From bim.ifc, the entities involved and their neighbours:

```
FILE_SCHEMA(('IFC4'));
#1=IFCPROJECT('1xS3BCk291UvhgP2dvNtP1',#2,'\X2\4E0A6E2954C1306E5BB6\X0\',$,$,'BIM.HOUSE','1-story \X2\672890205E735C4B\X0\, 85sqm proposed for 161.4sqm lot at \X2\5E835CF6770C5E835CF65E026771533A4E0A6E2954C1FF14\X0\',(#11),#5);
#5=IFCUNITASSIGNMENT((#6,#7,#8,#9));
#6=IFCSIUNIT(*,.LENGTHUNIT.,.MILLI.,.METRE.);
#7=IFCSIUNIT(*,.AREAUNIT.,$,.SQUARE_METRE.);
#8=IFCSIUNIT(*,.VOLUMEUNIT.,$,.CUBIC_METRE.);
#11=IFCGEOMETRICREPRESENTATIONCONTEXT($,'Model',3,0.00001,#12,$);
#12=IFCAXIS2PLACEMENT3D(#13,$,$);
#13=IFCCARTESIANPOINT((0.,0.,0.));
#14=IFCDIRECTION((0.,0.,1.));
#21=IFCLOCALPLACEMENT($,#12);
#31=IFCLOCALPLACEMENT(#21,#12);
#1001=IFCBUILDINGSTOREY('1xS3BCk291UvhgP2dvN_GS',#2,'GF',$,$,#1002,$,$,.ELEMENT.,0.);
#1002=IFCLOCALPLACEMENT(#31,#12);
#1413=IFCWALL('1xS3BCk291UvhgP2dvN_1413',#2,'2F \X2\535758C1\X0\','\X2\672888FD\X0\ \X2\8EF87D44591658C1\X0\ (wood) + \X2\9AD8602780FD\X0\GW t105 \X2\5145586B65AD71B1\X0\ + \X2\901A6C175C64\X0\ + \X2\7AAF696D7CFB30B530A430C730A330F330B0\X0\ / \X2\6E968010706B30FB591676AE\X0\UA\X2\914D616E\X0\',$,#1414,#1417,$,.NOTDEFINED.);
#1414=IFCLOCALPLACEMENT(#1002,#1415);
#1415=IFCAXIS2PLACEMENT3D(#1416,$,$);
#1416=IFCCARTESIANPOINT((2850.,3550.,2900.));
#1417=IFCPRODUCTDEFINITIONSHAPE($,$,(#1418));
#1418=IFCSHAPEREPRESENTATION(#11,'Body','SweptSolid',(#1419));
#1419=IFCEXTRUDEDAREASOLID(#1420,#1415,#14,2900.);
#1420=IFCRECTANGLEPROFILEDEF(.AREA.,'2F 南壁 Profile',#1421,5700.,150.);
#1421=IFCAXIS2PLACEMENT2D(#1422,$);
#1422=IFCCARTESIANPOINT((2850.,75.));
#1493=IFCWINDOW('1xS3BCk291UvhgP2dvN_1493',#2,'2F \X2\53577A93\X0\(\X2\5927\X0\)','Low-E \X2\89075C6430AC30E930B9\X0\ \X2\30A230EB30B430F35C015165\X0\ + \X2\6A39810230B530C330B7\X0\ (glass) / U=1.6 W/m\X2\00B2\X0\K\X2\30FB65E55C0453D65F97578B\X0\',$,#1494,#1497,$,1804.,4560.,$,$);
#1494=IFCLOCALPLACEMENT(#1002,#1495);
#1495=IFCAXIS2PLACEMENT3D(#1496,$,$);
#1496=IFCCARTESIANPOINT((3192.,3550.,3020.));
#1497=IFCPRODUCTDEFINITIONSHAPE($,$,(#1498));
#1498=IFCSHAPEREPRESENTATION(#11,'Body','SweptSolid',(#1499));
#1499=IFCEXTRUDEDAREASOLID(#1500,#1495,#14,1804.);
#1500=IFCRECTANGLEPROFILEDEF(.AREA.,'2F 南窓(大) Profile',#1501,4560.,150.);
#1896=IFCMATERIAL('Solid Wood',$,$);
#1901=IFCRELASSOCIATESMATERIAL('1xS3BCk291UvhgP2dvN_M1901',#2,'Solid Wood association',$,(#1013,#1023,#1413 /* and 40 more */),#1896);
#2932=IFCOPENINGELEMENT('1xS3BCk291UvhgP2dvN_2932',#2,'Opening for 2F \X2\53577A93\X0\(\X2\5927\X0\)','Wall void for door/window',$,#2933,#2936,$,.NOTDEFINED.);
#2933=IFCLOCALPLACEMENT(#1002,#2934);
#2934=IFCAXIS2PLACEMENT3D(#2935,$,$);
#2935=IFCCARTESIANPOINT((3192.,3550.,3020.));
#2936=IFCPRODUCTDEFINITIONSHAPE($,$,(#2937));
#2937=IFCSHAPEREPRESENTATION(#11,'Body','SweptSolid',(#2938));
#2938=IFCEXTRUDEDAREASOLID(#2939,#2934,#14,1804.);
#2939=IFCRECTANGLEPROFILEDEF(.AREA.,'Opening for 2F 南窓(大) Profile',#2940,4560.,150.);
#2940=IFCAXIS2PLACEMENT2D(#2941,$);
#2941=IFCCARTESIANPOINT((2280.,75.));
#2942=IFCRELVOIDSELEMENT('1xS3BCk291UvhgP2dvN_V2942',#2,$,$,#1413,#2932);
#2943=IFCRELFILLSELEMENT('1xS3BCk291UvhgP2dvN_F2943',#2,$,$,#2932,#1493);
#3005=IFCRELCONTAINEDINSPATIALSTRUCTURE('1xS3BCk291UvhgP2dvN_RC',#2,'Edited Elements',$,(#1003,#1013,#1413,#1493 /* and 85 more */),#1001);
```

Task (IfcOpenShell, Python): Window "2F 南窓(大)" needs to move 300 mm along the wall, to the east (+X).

```python
import ifcopenshell
import ifcopenshell.api.geometry
import ifcopenshell.util.placement

model = ifcopenshell.open("bim.ifc")

window = model.by_guid("1xS3BCk291UvhgP2dvN_1493")
opening = window.FillsVoids[0].RelatingOpeningElement
wall = opening.VoidsElements[0].RelatingBuildingElement

wall_matrix = ifcopenshell.util.placement.get_local_placement(wall.ObjectPlacement)
shift = wall_matrix[:3, 0] * 300.0
before = ifcopenshell.util.placement.get_local_placement(window.ObjectPlacement)[:3, 3].copy()

# The window is not placed relative to its opening, so move both.
for product in (opening, window):
    matrix = ifcopenshell.util.placement.get_local_placement(product.ObjectPlacement)
    matrix[:3, 3] += shift
    ifcopenshell.api.geometry.edit_object_placement(model, product=product, matrix=matrix, is_si=False)

after = ifcopenshell.util.placement.get_local_placement(window.ObjectPlacement)[:3, 3]
print("window moved by", (after - before).round(3) + 0.0)

model.write("bim_rev.ifc")
```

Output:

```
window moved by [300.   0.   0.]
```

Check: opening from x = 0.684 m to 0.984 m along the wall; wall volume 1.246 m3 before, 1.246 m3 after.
